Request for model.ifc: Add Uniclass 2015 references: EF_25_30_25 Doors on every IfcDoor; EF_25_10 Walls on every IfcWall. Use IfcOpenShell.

First a look at what the model holds.

```python
import ifcopenshell

model = ifcopenshell.open("model.ifc")
print(model.schema)
print("classifications:", [c.Name for c in model.by_type("IfcClassification")])
for ifc_class in ("IfcDoor", "IfcRoof", "IfcStair", "IfcWall", "IfcWindow"):
    print(ifc_class, len(model.by_type(ifc_class)))
```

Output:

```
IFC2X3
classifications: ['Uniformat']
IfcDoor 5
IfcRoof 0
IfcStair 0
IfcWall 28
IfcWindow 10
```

```python
import ifcopenshell
import ifcopenshell.api.classification

model = ifcopenshell.open("model.ifc")

# IFC2X3 requires Source and Edition and has no link from the project to the system.
system = model.create_entity("IfcClassification", Source="NBS", Edition="2015", Name="Uniclass 2015")

codes = {
    "IfcDoor": ("EF_25_30_25", "Doors"),
    "IfcWall": ("EF_25_10", "Walls"),
}
for ifc_class, (code, name) in codes.items():
    products = model.by_type(ifc_class)
    ifcopenshell.api.classification.add_reference(
        model, products=products, classification=system, identification=code, name=name
    )
    print(code, len(products))

model.write("model_edited.ifc")
```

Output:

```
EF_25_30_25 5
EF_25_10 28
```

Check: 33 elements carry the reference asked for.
